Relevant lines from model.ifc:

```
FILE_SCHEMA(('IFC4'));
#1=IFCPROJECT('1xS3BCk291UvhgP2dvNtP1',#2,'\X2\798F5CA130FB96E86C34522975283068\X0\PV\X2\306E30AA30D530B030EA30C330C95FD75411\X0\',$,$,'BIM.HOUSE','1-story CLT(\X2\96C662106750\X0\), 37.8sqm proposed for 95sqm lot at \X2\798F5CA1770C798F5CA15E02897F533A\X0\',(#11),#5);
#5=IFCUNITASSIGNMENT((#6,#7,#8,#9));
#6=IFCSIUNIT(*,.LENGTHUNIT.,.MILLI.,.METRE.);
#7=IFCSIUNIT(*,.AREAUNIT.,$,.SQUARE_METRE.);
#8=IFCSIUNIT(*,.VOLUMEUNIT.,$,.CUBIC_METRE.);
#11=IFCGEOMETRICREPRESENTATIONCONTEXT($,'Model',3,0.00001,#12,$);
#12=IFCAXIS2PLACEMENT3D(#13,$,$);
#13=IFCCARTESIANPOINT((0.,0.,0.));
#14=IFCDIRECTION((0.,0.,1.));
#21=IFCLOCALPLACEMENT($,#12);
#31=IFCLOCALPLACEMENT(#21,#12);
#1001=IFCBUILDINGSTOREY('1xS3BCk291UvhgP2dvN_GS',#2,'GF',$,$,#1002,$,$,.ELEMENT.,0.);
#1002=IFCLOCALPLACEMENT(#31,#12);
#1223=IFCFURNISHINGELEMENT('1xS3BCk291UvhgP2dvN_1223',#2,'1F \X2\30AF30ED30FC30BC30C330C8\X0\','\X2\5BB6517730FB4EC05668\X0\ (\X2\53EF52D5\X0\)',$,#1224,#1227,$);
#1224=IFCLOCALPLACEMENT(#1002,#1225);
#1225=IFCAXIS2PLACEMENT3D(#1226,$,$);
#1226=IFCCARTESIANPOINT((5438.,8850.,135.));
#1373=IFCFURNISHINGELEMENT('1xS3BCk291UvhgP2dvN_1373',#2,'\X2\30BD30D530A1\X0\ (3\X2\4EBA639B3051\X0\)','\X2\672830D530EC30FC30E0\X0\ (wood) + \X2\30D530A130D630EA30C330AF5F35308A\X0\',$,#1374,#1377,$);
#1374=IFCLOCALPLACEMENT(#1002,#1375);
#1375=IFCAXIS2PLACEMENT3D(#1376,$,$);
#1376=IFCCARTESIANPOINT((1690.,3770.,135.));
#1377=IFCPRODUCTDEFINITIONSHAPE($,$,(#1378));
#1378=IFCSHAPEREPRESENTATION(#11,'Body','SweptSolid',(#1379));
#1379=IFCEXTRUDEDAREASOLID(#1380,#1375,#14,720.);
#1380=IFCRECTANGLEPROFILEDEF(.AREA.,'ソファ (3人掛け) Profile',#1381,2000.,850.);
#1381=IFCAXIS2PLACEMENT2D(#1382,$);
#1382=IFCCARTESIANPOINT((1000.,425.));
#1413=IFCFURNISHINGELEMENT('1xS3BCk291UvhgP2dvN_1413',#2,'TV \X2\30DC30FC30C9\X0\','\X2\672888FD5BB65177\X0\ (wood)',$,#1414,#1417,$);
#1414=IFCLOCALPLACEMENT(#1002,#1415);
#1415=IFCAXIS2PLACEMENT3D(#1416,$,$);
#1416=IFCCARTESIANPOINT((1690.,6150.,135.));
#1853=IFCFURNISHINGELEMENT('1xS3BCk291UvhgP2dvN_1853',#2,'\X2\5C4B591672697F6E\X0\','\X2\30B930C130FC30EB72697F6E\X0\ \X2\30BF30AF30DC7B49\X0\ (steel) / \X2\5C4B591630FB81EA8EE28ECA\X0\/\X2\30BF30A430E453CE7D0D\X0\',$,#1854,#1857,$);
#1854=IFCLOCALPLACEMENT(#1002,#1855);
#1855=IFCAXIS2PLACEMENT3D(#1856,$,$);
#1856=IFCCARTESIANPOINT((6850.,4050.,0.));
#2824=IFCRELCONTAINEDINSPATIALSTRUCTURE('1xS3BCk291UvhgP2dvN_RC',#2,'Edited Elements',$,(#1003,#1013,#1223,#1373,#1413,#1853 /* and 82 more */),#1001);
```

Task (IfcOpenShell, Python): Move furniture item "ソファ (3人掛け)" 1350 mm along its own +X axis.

```python
import ifcopenshell
import ifcopenshell.api.geometry
import ifcopenshell.util.placement
import ifcopenshell.util.unit

model = ifcopenshell.open("model.ifc")
unit_scale = ifcopenshell.util.unit.calculate_unit_scale(model)

item = model.by_guid("1xS3BCk291UvhgP2dvN_1373")
matrix = ifcopenshell.util.placement.get_local_placement(item.ObjectPlacement)
matrix[:3, 3] += matrix[:3, 0] * 1.35 / unit_scale
ifcopenshell.api.geometry.edit_object_placement(model, product=item, matrix=matrix, is_si=False)

print(ifcopenshell.util.placement.get_local_placement(item.ObjectPlacement).round(3) + 0.0)

model.write("model_updated.ifc")
```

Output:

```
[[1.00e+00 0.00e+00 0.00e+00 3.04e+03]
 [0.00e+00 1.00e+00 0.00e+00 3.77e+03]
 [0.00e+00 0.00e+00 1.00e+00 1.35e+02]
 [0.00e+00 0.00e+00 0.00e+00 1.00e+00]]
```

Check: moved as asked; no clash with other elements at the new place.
